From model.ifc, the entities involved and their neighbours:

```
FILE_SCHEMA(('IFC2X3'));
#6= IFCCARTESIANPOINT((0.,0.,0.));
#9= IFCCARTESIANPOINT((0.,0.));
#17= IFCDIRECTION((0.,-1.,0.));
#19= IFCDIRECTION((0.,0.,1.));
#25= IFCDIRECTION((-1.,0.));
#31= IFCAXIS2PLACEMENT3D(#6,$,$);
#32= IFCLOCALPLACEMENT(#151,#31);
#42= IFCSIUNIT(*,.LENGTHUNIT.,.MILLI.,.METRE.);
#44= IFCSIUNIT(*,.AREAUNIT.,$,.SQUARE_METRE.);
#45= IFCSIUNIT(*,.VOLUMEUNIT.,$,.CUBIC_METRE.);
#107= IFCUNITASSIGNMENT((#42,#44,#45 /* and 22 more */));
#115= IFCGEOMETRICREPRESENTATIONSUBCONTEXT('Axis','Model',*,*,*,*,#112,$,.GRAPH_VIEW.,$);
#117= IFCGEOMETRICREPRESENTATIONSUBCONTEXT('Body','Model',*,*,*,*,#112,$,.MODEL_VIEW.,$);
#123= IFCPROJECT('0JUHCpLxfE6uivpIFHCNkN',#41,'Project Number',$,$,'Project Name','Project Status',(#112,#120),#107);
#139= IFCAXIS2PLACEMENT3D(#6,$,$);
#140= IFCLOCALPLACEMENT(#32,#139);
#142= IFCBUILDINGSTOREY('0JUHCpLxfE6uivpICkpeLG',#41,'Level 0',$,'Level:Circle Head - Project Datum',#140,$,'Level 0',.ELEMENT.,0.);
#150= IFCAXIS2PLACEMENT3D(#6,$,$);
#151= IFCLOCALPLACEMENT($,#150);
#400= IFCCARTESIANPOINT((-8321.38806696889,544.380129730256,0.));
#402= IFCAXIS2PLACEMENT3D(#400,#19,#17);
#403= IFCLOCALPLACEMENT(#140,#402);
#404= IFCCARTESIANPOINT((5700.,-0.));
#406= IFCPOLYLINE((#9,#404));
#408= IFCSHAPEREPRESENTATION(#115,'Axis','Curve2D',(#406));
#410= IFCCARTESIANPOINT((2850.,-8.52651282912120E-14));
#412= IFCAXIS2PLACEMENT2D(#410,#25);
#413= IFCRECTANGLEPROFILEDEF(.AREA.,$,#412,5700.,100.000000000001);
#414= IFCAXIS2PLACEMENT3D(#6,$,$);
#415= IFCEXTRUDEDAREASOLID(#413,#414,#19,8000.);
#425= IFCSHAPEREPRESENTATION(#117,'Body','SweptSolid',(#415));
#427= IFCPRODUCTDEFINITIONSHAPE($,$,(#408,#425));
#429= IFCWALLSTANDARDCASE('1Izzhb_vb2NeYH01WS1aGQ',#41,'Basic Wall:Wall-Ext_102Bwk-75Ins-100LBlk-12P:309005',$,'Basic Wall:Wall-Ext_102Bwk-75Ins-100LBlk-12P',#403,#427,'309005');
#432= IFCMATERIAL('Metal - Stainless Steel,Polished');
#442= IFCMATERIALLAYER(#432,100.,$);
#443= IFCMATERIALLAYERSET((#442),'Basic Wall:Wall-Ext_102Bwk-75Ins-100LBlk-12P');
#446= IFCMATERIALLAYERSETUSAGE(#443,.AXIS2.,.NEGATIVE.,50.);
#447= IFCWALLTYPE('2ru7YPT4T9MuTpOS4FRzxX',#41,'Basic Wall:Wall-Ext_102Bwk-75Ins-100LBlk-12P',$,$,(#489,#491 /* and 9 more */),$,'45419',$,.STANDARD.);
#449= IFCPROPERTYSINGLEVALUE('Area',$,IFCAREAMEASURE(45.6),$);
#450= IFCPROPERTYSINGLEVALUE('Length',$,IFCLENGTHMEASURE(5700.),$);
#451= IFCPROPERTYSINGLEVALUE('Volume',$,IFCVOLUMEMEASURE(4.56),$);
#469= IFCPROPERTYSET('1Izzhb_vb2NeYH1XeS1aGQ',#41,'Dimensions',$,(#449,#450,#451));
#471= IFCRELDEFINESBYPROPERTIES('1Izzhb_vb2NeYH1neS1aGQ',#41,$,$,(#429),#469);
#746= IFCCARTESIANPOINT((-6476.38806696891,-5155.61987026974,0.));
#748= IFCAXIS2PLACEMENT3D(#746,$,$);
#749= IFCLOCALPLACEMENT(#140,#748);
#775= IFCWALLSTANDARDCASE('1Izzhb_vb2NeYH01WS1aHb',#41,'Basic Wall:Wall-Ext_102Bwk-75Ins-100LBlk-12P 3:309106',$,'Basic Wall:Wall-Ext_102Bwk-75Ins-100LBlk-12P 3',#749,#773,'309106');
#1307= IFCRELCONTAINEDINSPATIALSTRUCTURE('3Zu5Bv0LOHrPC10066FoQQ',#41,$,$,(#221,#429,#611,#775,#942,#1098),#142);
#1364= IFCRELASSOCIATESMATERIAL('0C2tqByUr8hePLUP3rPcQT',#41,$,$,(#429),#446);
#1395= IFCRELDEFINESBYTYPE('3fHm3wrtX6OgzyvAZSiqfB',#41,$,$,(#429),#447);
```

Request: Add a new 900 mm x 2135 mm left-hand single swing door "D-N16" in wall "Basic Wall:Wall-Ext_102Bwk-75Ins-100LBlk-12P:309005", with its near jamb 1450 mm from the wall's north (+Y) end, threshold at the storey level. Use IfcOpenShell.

```python
import numpy as np
import ifcopenshell
import ifcopenshell.api.feature
import ifcopenshell.api.geometry
import ifcopenshell.api.pset
import ifcopenshell.api.root
import ifcopenshell.api.spatial
import ifcopenshell.api.type
import ifcopenshell.geom
import ifcopenshell.util.element
import ifcopenshell.util.placement
import ifcopenshell.util.representation
import ifcopenshell.util.shape
import ifcopenshell.util.unit

model = ifcopenshell.open("model.ifc")
unit_scale = ifcopenshell.util.unit.calculate_unit_scale(model)
area_scale = ifcopenshell.util.unit.calculate_unit_scale(model, "AREAUNIT")
volume_scale = ifcopenshell.util.unit.calculate_unit_scale(model, "VOLUMEUNIT")
settings = ifcopenshell.geom.settings()


def volume(element):
    """Net volume in cubic metres, openings subtracted."""
    shape = ifcopenshell.geom.create_shape(settings, element)
    return ifcopenshell.util.shape.get_volume(shape.geometry)


wall = model.by_id(429)
storey = ifcopenshell.util.element.get_container(wall, ifc_class="IfcBuildingStorey")
context = ifcopenshell.util.representation.get_context(model, "Model", "Body", "MODEL_VIEW")
before = volume(wall)

width, height, from_end, sill = 0.9, 2.135, 1.45, 0.0  # metres

# The wall runs along its own X axis, and the end named is its -X end.
wall_shape = ifcopenshell.geom.create_shape(settings, wall)
x, y, z = ifcopenshell.util.shape.get_vertices(wall_shape.geometry).T
start = x.min() + from_end
face, thickness = float(y.min()), float(y.max() - y.min())
wall_matrix = ifcopenshell.util.placement.get_local_placement(wall.ObjectPlacement)
level = ifcopenshell.util.placement.get_local_placement(storey.ObjectPlacement)[2, 3]


def in_wall(x, y):
    """Placement at x, y metres in the wall's axes, at sill height."""
    matrix = wall_matrix.copy()
    matrix[:, 3] = wall_matrix @ np.array([x / unit_scale, y / unit_scale, 0.0, 1.0])
    matrix[2, 3] = level + sill / unit_scale
    return matrix


# Opening: a box that overshoots both wall faces by 50 mm.
opening = ifcopenshell.api.root.create_entity(model, ifc_class="IfcOpeningElement")
box = ifcopenshell.api.geometry.add_wall_representation(
    model, context=context, length=width, height=height, thickness=thickness + 0.1
)
ifcopenshell.api.geometry.assign_representation(model, product=opening, representation=box)
ifcopenshell.api.geometry.edit_object_placement(model, product=opening, matrix=in_wall(start, face - 0.05), is_si=False)
ifcopenshell.api.feature.add_feature(model, feature=opening, element=wall)

door = ifcopenshell.api.root.create_entity(model, ifc_class="IfcDoor", name="D-N16")
door.OverallWidth, door.OverallHeight = width / unit_scale, height / unit_scale
body = ifcopenshell.api.geometry.add_door_representation(
    model,
    context=context,
    overall_width=door.OverallWidth,
    overall_height=door.OverallHeight,
    operation_type="SINGLE_SWING_LEFT",
    lining_properties={"LiningDepth": thickness / unit_scale, "ThresholdDepth": thickness / unit_scale},
)
ifcopenshell.api.geometry.assign_representation(model, product=door, representation=body)
ifcopenshell.api.spatial.assign_container(model, products=[door], relating_structure=storey)
fills = ifcopenshell.api.feature.add_filling(model, opening=opening, element=door)
fills.OwnerHistory = door.OwnerHistory  # required in IFC2X3

# IFC2X3 keeps the operation on the door style.
style = ifcopenshell.api.root.create_entity(model, ifc_class="IfcDoorStyle", name="D-N16")
style.OperationType, style.ConstructionType = "SINGLE_SWING_LEFT", "NOTDEFINED"
style.ParameterTakesPrecedence = style.Sizeable = False
ifcopenshell.api.type.assign_type(model, related_objects=[door], relating_type=style)

# The lining spans the wall, so the door starts at the wall face.
ifcopenshell.api.geometry.edit_object_placement(model, product=door, matrix=in_wall(start, face), is_si=False)

after = volume(wall)

# Update the wall's stored quantities.
pset = model.by_id(ifcopenshell.util.element.get_pset(wall, "Dimensions", should_inherit=False)["id"])
ifcopenshell.api.pset.edit_pset(model, pset=pset, properties={
    "Area": model.create_entity("IfcAreaMeasure", after / thickness / area_scale),
    "Volume": model.create_entity("IfcVolumeMeasure", after / volume_scale),
})

print(f"wall volume {before:.3f} -> {after:.3f} m3")

model.write("model_updated.ifc")
```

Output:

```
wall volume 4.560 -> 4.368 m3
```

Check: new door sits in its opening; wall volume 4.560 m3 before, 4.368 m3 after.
